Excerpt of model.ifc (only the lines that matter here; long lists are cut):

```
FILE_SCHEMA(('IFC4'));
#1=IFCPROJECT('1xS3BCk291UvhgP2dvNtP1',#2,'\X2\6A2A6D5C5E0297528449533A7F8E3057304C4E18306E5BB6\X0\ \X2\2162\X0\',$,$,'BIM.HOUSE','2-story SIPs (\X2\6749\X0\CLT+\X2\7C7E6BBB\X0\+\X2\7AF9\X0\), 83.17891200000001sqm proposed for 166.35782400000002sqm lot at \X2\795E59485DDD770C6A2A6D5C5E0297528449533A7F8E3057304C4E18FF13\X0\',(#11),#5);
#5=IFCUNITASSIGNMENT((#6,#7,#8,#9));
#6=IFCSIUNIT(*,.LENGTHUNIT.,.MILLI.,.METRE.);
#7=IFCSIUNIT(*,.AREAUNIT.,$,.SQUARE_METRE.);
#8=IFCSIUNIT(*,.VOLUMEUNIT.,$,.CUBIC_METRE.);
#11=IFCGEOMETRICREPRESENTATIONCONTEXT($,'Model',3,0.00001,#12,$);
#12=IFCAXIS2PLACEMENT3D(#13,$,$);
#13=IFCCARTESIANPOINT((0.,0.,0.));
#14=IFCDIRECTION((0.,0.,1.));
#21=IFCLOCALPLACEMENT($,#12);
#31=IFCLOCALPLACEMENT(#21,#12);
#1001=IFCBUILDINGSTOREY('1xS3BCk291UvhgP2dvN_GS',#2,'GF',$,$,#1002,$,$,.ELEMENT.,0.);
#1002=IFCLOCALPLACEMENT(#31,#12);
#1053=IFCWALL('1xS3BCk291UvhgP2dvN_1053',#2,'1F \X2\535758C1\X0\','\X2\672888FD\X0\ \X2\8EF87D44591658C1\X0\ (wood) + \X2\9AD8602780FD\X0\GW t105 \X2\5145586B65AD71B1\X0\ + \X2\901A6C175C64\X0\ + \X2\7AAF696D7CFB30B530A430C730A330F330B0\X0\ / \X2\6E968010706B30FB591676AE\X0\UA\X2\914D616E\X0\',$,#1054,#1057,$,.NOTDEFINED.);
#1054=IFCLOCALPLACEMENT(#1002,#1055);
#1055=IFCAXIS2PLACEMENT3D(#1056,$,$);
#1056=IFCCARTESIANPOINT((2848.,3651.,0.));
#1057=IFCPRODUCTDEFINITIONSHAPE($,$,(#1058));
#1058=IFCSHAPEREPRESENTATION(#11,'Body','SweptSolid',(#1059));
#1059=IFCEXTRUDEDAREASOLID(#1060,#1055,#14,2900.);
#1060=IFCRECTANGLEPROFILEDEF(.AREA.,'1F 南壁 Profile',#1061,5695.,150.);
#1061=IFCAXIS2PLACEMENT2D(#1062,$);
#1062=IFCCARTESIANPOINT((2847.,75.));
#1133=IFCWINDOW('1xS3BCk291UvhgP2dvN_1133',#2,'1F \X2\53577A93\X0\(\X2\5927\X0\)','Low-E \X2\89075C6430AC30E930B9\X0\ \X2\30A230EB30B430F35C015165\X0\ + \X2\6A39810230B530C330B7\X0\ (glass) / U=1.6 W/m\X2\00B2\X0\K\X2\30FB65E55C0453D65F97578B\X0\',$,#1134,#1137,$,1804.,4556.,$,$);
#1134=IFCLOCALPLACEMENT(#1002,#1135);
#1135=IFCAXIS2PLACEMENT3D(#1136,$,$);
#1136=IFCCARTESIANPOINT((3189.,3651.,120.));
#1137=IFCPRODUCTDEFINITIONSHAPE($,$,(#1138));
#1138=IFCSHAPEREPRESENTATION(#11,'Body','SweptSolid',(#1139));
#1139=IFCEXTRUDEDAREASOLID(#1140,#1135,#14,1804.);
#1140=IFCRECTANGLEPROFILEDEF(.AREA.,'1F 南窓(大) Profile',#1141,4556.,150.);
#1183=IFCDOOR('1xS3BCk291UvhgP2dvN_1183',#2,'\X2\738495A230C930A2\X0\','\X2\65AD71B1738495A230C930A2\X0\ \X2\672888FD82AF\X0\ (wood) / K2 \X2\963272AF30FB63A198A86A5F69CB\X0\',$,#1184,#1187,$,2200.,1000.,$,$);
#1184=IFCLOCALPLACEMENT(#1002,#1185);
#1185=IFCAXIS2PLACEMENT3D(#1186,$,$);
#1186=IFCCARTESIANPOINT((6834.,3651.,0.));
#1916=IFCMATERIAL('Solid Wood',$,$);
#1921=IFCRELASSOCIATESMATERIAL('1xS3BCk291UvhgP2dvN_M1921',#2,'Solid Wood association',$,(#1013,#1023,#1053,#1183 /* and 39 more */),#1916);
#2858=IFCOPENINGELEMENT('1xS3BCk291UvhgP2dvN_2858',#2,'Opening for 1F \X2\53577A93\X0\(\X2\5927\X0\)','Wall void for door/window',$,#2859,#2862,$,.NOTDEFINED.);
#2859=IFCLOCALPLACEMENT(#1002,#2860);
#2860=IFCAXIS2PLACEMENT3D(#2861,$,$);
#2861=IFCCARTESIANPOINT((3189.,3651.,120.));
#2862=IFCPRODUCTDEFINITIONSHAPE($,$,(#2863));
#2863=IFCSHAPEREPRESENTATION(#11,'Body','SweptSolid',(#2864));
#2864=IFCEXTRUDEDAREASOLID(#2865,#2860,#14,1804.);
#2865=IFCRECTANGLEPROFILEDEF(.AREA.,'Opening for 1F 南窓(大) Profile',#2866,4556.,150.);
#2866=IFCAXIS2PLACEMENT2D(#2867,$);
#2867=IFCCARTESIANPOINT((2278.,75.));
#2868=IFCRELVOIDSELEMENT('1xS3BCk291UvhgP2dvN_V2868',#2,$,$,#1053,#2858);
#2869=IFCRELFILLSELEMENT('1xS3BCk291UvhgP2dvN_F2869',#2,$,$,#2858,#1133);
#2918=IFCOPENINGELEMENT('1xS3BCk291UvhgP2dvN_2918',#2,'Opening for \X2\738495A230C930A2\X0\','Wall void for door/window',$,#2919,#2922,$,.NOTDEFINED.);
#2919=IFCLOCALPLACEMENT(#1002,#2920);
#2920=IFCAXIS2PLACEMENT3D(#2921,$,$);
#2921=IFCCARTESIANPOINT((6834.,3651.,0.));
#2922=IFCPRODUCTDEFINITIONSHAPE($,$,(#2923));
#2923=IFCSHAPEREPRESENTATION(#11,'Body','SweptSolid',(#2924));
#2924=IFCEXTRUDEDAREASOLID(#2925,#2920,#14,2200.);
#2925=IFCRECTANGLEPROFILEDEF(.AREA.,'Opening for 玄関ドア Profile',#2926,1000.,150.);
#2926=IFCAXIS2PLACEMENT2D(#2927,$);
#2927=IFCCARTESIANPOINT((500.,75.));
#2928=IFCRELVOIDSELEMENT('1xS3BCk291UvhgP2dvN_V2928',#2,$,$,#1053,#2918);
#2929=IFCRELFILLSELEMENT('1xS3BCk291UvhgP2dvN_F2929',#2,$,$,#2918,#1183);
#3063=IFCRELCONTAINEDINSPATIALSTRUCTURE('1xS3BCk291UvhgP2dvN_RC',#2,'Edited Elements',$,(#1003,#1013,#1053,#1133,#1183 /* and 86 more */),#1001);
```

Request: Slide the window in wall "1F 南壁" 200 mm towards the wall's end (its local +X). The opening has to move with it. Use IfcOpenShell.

```python
import ifcopenshell
import ifcopenshell.api.geometry
import ifcopenshell.util.placement
import ifcopenshell.util.unit

model = ifcopenshell.open("model.ifc")
unit_scale = ifcopenshell.util.unit.calculate_unit_scale(model)

window = model.by_guid("1xS3BCk291UvhgP2dvN_1133")
opening = window.FillsVoids[0].RelatingOpeningElement
wall = opening.VoidsElements[0].RelatingBuildingElement

wall_matrix = ifcopenshell.util.placement.get_local_placement(wall.ObjectPlacement)
shift = wall_matrix[:3, 0] * 0.2 / unit_scale
before = ifcopenshell.util.placement.get_local_placement(window.ObjectPlacement)[:3, 3].copy()

# The window is not placed relative to its opening, so move both.
for product in (opening, window):
    matrix = ifcopenshell.util.placement.get_local_placement(product.ObjectPlacement)
    matrix[:3, 3] += shift
    ifcopenshell.api.geometry.edit_object_placement(model, product=product, matrix=matrix, is_si=False)

after = ifcopenshell.util.placement.get_local_placement(window.ObjectPlacement)[:3, 3]
print("window moved by", (after - before).round(3) + 0.0)

model.write("model_rev.ifc")
```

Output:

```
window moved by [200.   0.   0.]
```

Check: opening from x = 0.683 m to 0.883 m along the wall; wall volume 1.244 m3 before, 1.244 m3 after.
